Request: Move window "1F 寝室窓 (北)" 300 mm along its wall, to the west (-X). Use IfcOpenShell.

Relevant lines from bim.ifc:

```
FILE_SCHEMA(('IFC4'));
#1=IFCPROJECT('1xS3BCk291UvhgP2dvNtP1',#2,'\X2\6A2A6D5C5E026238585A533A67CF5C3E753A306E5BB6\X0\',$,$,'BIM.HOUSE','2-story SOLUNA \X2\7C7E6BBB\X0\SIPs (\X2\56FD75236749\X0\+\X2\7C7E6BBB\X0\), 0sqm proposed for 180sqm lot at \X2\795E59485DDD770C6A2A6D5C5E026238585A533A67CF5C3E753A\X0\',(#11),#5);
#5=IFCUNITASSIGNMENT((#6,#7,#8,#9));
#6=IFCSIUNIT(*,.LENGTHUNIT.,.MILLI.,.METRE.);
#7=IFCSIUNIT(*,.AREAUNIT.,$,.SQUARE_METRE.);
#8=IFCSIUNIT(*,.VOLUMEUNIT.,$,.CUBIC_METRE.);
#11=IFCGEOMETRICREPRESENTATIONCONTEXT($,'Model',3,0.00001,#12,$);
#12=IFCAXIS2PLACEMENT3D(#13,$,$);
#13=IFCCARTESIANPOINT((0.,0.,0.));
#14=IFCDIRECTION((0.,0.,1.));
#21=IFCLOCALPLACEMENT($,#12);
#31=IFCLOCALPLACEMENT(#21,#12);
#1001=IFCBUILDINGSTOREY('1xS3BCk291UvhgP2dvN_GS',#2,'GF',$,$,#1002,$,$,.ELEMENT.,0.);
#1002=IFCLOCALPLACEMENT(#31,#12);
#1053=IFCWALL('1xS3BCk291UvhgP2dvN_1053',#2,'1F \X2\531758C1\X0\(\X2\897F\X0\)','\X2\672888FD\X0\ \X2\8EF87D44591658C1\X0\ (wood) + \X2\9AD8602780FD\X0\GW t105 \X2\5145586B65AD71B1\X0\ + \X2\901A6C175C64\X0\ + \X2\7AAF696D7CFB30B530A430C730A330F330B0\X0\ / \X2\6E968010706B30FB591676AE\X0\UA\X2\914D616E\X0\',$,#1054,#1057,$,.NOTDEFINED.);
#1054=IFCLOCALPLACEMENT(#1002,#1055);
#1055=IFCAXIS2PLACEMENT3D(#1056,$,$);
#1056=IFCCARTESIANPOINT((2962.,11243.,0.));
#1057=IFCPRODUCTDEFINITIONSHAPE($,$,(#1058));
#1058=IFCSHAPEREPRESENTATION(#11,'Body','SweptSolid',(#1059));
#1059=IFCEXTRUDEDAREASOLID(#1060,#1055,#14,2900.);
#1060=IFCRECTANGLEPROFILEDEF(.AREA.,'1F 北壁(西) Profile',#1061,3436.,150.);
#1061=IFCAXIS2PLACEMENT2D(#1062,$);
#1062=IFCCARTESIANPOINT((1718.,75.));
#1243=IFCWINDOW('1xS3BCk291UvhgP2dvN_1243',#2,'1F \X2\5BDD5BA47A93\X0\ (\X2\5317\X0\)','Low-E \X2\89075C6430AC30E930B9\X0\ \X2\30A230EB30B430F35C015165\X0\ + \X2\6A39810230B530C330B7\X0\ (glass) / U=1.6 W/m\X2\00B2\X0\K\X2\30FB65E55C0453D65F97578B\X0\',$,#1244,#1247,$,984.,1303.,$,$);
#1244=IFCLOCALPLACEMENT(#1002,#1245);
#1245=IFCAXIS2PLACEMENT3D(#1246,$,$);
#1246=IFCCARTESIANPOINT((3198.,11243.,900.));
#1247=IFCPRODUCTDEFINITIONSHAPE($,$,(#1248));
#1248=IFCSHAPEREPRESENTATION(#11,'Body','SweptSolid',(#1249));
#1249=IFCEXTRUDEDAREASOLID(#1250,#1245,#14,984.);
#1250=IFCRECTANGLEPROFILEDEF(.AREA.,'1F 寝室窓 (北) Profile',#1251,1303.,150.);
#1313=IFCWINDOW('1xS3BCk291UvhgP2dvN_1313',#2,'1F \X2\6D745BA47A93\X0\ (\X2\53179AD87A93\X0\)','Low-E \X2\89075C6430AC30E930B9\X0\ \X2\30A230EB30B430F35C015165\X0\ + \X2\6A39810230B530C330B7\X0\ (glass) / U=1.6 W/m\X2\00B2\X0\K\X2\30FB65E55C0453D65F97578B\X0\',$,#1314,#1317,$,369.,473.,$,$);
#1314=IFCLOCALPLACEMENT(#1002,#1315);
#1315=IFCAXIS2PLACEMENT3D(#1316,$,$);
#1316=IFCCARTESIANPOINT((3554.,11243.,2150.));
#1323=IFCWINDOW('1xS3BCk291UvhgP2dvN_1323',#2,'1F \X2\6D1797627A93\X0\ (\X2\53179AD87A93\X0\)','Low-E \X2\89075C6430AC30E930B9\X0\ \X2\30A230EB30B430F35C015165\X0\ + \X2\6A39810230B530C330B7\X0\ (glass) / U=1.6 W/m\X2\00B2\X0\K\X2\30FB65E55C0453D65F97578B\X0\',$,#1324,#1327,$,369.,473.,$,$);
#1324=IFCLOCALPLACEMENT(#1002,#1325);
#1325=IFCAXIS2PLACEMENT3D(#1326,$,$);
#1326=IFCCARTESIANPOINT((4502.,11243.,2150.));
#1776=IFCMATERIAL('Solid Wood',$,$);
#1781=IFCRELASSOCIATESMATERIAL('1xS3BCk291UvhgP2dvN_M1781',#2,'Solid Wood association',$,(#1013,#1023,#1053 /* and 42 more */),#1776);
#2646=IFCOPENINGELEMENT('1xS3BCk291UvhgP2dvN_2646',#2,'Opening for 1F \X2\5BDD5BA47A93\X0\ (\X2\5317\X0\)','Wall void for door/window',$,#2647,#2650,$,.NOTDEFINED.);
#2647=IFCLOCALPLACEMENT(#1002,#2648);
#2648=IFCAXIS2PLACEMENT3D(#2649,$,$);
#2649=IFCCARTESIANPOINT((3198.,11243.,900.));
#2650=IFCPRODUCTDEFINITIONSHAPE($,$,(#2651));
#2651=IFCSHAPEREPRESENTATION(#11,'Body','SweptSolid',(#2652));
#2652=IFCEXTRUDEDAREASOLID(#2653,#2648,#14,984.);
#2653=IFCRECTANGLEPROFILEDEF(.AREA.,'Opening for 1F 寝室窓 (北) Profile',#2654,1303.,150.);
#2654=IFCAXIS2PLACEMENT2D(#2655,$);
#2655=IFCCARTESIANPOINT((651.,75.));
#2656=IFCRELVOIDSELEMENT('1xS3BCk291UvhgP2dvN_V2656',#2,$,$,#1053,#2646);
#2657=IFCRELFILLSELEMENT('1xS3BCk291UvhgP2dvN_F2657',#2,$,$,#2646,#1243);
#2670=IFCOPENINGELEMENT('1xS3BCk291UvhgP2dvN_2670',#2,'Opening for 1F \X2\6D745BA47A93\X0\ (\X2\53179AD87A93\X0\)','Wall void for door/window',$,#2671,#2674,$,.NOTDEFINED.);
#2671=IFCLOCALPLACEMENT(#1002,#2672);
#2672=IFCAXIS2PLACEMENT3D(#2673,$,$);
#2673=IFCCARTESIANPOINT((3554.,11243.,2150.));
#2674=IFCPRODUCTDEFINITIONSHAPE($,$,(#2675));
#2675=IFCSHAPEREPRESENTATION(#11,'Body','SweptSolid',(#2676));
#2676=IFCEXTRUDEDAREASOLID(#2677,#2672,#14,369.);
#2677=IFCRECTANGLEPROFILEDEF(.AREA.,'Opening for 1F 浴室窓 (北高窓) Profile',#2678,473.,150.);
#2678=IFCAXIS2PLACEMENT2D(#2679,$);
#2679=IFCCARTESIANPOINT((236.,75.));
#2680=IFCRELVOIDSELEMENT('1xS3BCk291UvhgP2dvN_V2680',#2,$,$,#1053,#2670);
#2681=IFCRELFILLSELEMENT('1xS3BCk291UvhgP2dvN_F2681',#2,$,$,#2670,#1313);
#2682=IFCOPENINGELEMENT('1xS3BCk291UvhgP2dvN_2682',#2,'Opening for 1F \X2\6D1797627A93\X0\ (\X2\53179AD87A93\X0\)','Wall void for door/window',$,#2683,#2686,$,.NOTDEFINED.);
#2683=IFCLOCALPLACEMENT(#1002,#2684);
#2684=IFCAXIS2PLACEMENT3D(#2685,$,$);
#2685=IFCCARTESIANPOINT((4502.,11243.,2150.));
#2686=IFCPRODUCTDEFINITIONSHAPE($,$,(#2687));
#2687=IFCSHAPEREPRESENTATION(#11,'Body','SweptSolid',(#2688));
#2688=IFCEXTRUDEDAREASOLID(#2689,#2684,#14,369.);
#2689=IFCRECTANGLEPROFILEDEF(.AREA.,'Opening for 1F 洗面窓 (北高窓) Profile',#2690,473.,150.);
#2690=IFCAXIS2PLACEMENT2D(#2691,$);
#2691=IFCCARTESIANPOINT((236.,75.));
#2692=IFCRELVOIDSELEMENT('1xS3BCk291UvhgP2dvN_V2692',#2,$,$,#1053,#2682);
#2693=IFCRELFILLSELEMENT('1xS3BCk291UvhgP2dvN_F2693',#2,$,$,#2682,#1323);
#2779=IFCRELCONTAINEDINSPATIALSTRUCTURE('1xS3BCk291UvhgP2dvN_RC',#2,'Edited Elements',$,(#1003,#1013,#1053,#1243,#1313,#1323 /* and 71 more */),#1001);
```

```python
import ifcopenshell
import ifcopenshell.api.geometry
import ifcopenshell.util.placement

model = ifcopenshell.open("bim.ifc")

window = model.by_guid("1xS3BCk291UvhgP2dvN_1243")
opening = window.FillsVoids[0].RelatingOpeningElement
wall = opening.VoidsElements[0].RelatingBuildingElement

wall_matrix = ifcopenshell.util.placement.get_local_placement(wall.ObjectPlacement)
shift = wall_matrix[:3, 0] * -300.0
before = ifcopenshell.util.placement.get_local_placement(window.ObjectPlacement)[:3, 3].copy()

# The window is not placed relative to its opening, so move both.
for product in (opening, window):
    matrix = ifcopenshell.util.placement.get_local_placement(product.ObjectPlacement)
    matrix[:3, 3] += shift
    ifcopenshell.api.geometry.edit_object_placement(model, product=product, matrix=matrix, is_si=False)

after = ifcopenshell.util.placement.get_local_placement(window.ObjectPlacement)[:3, 3]
print("window moved by", (after - before).round(3) + 0.0)

model.write("bim_v2.ifc")
```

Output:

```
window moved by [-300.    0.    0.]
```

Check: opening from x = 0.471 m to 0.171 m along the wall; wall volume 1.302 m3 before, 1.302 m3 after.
